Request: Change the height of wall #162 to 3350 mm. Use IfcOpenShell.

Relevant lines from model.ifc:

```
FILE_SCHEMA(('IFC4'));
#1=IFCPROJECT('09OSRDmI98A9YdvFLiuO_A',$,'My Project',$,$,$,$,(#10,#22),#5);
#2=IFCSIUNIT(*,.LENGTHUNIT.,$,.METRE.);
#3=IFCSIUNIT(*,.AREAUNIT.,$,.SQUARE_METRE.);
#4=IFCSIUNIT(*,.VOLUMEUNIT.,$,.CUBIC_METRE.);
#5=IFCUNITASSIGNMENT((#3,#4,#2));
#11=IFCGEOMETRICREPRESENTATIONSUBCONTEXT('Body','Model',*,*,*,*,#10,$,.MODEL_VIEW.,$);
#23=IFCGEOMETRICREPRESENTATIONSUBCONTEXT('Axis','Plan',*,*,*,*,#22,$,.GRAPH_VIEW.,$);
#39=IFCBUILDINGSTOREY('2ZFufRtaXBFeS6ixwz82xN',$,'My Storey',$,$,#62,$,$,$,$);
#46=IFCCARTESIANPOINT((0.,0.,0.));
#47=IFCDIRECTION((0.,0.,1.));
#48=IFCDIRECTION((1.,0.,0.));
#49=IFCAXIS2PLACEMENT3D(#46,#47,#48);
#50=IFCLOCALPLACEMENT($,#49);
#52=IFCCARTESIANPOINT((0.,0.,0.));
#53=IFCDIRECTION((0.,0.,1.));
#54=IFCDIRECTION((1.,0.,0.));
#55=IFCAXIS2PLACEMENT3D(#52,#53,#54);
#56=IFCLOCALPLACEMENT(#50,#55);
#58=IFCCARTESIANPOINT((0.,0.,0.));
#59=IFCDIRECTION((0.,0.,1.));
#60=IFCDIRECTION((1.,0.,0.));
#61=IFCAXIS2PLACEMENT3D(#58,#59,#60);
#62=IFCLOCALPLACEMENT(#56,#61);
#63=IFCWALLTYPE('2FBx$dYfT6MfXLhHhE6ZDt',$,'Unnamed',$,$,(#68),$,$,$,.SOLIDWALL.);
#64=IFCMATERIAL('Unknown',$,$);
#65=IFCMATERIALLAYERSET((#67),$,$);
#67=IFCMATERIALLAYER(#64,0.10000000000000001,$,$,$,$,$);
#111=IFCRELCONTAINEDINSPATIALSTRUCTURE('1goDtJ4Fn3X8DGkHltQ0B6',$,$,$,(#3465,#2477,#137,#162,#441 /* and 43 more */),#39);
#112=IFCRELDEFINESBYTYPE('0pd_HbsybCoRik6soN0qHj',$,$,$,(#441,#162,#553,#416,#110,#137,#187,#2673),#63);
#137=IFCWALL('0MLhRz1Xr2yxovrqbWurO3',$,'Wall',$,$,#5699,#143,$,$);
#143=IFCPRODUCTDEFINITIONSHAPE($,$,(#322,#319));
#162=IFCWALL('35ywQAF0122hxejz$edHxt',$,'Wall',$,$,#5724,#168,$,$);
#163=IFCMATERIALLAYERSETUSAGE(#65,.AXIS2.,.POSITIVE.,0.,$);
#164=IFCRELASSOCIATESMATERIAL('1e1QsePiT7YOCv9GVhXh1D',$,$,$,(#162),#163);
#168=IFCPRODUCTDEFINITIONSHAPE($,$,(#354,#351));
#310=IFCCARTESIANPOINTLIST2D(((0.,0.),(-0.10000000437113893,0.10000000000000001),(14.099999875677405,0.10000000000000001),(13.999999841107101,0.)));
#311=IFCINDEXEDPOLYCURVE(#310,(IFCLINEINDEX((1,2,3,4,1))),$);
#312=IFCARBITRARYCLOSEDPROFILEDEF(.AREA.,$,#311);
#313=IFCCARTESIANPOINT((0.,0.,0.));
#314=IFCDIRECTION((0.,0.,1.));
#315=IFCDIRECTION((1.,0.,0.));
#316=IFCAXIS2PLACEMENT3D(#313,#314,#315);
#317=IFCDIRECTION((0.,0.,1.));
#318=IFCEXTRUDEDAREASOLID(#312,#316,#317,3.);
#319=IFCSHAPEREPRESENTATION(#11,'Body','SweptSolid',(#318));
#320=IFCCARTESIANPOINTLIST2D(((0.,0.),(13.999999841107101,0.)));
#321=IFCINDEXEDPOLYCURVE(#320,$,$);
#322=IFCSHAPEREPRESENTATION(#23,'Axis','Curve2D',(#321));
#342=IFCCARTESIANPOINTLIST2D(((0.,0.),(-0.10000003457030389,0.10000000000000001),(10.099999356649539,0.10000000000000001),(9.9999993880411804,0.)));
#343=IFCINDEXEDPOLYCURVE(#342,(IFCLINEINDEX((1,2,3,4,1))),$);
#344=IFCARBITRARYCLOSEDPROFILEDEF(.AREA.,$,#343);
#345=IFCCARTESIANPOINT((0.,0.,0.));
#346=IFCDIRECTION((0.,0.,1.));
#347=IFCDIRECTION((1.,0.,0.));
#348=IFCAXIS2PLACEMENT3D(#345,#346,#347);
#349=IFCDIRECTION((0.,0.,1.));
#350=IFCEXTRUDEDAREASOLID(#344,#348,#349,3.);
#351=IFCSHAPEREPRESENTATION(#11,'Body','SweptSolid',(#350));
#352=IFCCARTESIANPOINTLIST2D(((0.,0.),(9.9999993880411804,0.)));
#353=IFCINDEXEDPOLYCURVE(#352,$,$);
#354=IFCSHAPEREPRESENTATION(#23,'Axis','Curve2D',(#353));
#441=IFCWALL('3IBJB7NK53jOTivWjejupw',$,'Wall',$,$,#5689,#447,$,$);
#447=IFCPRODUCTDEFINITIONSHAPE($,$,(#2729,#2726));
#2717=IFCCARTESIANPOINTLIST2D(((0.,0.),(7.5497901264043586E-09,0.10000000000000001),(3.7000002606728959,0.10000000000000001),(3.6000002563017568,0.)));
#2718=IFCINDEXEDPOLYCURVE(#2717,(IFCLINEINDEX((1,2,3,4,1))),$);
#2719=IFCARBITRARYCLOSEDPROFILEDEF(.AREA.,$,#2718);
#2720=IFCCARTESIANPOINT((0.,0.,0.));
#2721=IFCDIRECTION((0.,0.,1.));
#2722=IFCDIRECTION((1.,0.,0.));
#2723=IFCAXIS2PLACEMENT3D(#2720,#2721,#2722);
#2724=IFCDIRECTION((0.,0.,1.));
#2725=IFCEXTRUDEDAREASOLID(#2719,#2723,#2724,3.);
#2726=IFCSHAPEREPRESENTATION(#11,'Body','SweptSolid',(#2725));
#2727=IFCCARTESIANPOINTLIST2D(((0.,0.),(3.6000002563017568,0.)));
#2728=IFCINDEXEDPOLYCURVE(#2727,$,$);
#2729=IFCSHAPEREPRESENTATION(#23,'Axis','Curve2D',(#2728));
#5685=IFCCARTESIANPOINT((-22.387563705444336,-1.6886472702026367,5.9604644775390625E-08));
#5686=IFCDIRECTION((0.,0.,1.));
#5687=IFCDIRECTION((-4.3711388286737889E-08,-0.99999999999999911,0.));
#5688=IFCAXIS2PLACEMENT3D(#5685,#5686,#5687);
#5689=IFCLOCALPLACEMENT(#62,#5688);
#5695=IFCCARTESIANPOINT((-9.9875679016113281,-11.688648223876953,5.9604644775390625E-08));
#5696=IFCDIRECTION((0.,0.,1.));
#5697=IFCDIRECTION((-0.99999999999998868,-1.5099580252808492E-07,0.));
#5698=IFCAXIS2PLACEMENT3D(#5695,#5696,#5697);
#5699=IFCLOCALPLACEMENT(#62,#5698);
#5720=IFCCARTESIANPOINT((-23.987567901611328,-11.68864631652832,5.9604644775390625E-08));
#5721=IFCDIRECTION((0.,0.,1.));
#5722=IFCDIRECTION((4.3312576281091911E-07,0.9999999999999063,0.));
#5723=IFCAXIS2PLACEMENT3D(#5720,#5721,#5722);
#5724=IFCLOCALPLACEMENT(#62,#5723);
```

```python
import ifcopenshell
import ifcopenshell.geom
import ifcopenshell.util.representation
import ifcopenshell.util.shape
import ifcopenshell.util.unit

model = ifcopenshell.open("model.ifc")
unit_scale = ifcopenshell.util.unit.calculate_unit_scale(model)
settings = ifcopenshell.geom.settings()


def volume(element):
    """Net volume in cubic metres, openings subtracted."""
    shape = ifcopenshell.geom.create_shape(settings, element)
    return ifcopenshell.util.shape.get_volume(shape.geometry)


wall = model.by_id(162)
before = volume(wall)

body = ifcopenshell.util.representation.get_representation(wall, "Model", "Body")
solid = body.Items[0]
old_height = solid.Depth
solid.Depth = 3.35 / unit_scale
after = volume(wall)

print(f"height {old_height:g} -> {solid.Depth:g}, volume {before:.3f} -> {after:.3f} m3")

model.write("model_rev.ifc")
```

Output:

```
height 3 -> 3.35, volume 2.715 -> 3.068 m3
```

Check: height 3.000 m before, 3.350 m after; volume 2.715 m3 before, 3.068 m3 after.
